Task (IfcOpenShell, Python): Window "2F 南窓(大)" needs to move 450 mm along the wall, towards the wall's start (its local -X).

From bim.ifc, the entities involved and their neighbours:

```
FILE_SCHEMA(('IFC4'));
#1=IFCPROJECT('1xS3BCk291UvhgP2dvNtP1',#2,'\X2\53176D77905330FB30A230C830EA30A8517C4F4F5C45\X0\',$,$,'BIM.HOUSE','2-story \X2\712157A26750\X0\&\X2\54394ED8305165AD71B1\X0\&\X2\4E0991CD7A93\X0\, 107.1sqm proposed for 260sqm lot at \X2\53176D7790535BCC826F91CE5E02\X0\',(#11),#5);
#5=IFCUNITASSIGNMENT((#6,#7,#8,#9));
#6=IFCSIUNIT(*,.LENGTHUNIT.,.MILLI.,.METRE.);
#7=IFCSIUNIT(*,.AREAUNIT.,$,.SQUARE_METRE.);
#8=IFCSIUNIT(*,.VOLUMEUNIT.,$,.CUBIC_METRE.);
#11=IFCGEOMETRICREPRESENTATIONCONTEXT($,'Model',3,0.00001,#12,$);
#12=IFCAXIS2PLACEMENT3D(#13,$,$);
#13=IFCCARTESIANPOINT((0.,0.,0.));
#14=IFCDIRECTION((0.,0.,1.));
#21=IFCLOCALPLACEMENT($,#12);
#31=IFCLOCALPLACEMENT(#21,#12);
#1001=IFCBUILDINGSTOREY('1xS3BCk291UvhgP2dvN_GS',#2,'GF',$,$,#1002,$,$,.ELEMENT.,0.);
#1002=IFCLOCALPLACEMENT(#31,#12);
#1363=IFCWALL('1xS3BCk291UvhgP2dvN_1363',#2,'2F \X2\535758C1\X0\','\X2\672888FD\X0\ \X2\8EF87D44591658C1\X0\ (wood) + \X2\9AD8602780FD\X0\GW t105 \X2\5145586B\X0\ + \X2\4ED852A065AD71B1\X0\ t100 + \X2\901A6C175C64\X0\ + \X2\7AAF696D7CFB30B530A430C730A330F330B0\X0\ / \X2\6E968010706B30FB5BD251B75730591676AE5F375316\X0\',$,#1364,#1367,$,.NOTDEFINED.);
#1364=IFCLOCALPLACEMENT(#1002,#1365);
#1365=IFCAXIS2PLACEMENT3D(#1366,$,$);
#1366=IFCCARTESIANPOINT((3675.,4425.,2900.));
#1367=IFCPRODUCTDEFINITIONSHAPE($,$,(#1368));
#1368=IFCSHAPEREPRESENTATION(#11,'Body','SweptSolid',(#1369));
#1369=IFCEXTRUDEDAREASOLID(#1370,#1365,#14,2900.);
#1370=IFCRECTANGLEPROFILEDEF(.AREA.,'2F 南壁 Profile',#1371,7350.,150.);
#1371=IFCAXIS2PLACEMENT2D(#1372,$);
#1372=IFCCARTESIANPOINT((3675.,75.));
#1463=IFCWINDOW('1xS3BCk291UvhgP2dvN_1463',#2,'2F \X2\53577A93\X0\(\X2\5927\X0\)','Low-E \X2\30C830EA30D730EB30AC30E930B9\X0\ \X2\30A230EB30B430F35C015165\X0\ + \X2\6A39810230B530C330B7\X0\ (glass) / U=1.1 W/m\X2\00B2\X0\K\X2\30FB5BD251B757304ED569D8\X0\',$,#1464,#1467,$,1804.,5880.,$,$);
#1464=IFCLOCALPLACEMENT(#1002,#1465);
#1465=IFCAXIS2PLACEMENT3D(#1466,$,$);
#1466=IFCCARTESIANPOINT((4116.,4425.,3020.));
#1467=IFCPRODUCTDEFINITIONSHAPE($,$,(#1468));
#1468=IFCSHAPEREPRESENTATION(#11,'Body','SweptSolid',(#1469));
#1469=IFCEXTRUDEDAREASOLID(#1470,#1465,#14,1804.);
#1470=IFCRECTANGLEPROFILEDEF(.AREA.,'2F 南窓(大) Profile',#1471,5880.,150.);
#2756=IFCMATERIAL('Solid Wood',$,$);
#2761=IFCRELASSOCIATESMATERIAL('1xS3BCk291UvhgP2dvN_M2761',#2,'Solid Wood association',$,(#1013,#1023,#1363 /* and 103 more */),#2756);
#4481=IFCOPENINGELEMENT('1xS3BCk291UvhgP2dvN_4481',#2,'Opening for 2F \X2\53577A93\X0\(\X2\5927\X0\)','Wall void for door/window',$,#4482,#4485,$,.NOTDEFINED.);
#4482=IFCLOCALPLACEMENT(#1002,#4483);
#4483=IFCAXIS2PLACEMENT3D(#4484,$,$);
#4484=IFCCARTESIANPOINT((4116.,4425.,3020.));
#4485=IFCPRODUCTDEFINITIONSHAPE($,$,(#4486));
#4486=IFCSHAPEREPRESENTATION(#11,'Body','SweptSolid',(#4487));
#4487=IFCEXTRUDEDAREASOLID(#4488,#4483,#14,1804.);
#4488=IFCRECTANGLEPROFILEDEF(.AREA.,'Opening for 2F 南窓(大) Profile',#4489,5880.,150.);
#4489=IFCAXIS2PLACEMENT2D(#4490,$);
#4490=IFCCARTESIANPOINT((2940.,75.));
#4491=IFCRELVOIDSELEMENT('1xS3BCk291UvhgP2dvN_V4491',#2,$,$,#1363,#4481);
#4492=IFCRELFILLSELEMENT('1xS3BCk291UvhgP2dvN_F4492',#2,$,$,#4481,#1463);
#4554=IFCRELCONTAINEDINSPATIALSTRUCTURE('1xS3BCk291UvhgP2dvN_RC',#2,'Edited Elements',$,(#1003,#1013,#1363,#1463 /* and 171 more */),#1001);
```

```python
import ifcopenshell
import ifcopenshell.api.geometry
import ifcopenshell.util.placement
import ifcopenshell.util.unit

model = ifcopenshell.open("bim.ifc")
unit_scale = ifcopenshell.util.unit.calculate_unit_scale(model)

window = model.by_guid("1xS3BCk291UvhgP2dvN_1463")
opening = window.FillsVoids[0].RelatingOpeningElement
wall = opening.VoidsElements[0].RelatingBuildingElement

wall_matrix = ifcopenshell.util.placement.get_local_placement(wall.ObjectPlacement)
shift = wall_matrix[:3, 0] * -0.45 / unit_scale
before = ifcopenshell.util.placement.get_local_placement(window.ObjectPlacement)[:3, 3].copy()

# The window is not placed relative to its opening, so move both.
for product in (opening, window):
    matrix = ifcopenshell.util.placement.get_local_placement(product.ObjectPlacement)
    matrix[:3, 3] += shift
    ifcopenshell.api.geometry.edit_object_placement(model, product=product, matrix=matrix, is_si=False)

after = ifcopenshell.util.placement.get_local_placement(window.ObjectPlacement)[:3, 3]
print("window moved by", (after - before).round(3) + 0.0)

model.write("bim_rev.ifc")
```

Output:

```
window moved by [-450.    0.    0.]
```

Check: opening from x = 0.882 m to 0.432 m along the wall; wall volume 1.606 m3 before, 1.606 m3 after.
